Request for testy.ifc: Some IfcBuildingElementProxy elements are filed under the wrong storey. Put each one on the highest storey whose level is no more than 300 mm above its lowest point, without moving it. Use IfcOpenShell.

First a look at what the model holds.

```python
import ifcopenshell
import ifcopenshell.util.element
import ifcopenshell.util.placement

model = ifcopenshell.open("testy.ifc")
print(model.schema)
for storey in model.by_type("IfcBuildingStorey"):
    level = ifcopenshell.util.placement.get_storey_elevation(storey)
    count = sum(e.is_a("IfcBuildingElementProxy") for e in ifcopenshell.util.element.get_contained(storey))
    print(storey.id(), storey.Name, round(level, 3), count, sep=" | ")
```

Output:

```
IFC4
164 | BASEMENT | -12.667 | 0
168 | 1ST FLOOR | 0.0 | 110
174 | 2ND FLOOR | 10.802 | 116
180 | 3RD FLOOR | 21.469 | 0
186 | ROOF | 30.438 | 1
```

```python
import ifcopenshell
import ifcopenshell.api.spatial
import ifcopenshell.geom
import ifcopenshell.util.element
import ifcopenshell.util.placement
import ifcopenshell.util.shape
import ifcopenshell.util.unit

model = ifcopenshell.open("testy.ifc")
unit_scale = ifcopenshell.util.unit.calculate_unit_scale(model)
settings = ifcopenshell.geom.settings()

levels = sorted(
    ((ifcopenshell.util.placement.get_storey_elevation(s) * unit_scale, s) for s in model.by_type("IfcBuildingStorey")),
    key=lambda pair: pair[0],
)

for e in model.by_type("IfcBuildingElementProxy"):
    current = e.ContainedInStructure[0].RelatingStructure if e.ContainedInStructure else None
    if current is None or not current.is_a("IfcBuildingStorey"):
        continue
    shape = ifcopenshell.geom.create_shape(settings, e)
    bottom = ifcopenshell.util.shape.get_shape_bottom_elevation(shape, shape.geometry)
    below = [s for level, s in levels if level <= bottom + 0.3]
    storey = below[-1] if below else levels[0][1]
    if storey != current:
        # assign_container keeps the world position.
        ifcopenshell.api.spatial.assign_container(model, products=[e], relating_structure=storey)
        print(e.id(), current.Name, "->", storey.Name)

model.write("testy_edited.ifc")
```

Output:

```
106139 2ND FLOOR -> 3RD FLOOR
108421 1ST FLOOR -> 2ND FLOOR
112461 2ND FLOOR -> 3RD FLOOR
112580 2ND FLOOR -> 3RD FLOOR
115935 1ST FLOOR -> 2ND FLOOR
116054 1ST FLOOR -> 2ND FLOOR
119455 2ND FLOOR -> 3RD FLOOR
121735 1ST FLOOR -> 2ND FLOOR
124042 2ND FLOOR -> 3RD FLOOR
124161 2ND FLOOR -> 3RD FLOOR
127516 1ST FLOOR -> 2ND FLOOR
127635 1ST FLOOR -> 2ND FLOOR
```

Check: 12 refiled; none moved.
